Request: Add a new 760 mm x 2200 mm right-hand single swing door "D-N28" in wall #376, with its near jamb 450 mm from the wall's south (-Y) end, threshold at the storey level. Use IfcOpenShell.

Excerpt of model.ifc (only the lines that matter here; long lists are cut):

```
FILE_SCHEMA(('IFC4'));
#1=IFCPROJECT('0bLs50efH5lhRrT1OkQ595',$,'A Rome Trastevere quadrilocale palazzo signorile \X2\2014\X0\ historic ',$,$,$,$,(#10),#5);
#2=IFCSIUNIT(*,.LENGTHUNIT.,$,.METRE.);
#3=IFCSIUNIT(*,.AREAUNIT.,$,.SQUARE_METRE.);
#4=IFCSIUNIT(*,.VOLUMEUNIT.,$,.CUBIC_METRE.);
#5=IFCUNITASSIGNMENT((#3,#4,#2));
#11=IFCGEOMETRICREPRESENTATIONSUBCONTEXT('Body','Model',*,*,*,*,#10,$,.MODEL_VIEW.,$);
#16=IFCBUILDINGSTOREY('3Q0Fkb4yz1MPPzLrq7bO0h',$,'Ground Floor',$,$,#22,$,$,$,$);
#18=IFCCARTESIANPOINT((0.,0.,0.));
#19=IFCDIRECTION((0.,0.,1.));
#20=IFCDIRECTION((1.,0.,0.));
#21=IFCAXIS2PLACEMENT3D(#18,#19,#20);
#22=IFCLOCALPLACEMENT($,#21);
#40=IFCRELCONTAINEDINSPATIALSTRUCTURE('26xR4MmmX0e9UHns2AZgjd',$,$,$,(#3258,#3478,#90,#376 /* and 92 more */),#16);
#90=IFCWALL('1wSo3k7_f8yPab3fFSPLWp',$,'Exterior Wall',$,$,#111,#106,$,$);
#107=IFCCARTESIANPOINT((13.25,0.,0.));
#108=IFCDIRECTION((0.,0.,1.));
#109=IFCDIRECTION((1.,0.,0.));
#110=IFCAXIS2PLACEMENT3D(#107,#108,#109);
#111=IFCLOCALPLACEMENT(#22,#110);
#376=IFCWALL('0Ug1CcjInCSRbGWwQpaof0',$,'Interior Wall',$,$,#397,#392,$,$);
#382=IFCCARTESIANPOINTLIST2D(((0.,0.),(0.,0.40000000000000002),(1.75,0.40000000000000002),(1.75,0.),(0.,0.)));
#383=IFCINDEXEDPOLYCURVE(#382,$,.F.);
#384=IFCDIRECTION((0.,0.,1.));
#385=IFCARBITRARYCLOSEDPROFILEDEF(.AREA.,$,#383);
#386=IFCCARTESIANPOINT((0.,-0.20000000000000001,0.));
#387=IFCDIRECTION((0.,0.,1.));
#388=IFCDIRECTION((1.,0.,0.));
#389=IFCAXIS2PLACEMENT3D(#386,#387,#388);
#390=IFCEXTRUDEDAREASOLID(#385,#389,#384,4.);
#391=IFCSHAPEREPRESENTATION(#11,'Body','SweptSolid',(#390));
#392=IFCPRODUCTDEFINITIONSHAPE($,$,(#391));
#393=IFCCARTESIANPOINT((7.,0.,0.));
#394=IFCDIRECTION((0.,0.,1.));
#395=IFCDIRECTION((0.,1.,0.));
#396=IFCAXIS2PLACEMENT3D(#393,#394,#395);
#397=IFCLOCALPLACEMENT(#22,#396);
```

```python
import numpy as np
import ifcopenshell
import ifcopenshell.api.feature
import ifcopenshell.api.geometry
import ifcopenshell.api.root
import ifcopenshell.api.spatial
import ifcopenshell.geom
import ifcopenshell.util.element
import ifcopenshell.util.placement
import ifcopenshell.util.representation
import ifcopenshell.util.shape
import ifcopenshell.util.unit

model = ifcopenshell.open("model.ifc")
unit_scale = ifcopenshell.util.unit.calculate_unit_scale(model)
settings = ifcopenshell.geom.settings()


def volume(element):
    """Net volume in cubic metres, openings subtracted."""
    shape = ifcopenshell.geom.create_shape(settings, element)
    return ifcopenshell.util.shape.get_volume(shape.geometry)


wall = model.by_guid("0Ug1CcjInCSRbGWwQpaof0")
storey = ifcopenshell.util.element.get_container(wall, ifc_class="IfcBuildingStorey")
context = ifcopenshell.util.representation.get_context(model, "Model", "Body", "MODEL_VIEW")
before = volume(wall)

width, height, from_end, sill = 0.76, 2.2, 0.45, 0.0  # metres

# The wall runs along its own X axis, and the end named is its -X end.
wall_shape = ifcopenshell.geom.create_shape(settings, wall)
x, y, z = ifcopenshell.util.shape.get_vertices(wall_shape.geometry).T
start = x.min() + from_end
face, thickness = float(y.min()), float(y.max() - y.min())
wall_matrix = ifcopenshell.util.placement.get_local_placement(wall.ObjectPlacement)
level = ifcopenshell.util.placement.get_local_placement(storey.ObjectPlacement)[2, 3]


def in_wall(x, y):
    """Placement at x, y metres in the wall's axes, at sill height."""
    matrix = wall_matrix.copy()
    matrix[:, 3] = wall_matrix @ np.array([x / unit_scale, y / unit_scale, 0.0, 1.0])
    matrix[2, 3] = level + sill / unit_scale
    return matrix


# Opening: a box that overshoots both wall faces by 50 mm.
opening = ifcopenshell.api.root.create_entity(model, ifc_class="IfcOpeningElement", predefined_type="OPENING")
box = ifcopenshell.api.geometry.add_wall_representation(
    model, context=context, length=width, height=height, thickness=thickness + 0.1
)
ifcopenshell.api.geometry.assign_representation(model, product=opening, representation=box)
ifcopenshell.api.geometry.edit_object_placement(model, product=opening, matrix=in_wall(start, face - 0.05), is_si=False)
ifcopenshell.api.feature.add_feature(model, feature=opening, element=wall)

door = ifcopenshell.api.root.create_entity(model, ifc_class="IfcDoor", name="D-N28", predefined_type="DOOR")
door.OverallWidth, door.OverallHeight = width / unit_scale, height / unit_scale
door.OperationType = "SINGLE_SWING_RIGHT"
body = ifcopenshell.api.geometry.add_door_representation(
    model,
    context=context,
    overall_width=door.OverallWidth,
    overall_height=door.OverallHeight,
    operation_type="SINGLE_SWING_RIGHT",
    lining_properties={"LiningDepth": thickness / unit_scale, "ThresholdDepth": thickness / unit_scale},
)
ifcopenshell.api.geometry.assign_representation(model, product=door, representation=body)
ifcopenshell.api.spatial.assign_container(model, products=[door], relating_structure=storey)
ifcopenshell.api.feature.add_filling(model, opening=opening, element=door)

# The lining spans the wall, so the door starts at the wall face.
ifcopenshell.api.geometry.edit_object_placement(model, product=door, matrix=in_wall(start, face), is_si=False)

after = volume(wall)

print(f"wall volume {before:.3f} -> {after:.3f} m3")

model.write("model_rev.ifc")
```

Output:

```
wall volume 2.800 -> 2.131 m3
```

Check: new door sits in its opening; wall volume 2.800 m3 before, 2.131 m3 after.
